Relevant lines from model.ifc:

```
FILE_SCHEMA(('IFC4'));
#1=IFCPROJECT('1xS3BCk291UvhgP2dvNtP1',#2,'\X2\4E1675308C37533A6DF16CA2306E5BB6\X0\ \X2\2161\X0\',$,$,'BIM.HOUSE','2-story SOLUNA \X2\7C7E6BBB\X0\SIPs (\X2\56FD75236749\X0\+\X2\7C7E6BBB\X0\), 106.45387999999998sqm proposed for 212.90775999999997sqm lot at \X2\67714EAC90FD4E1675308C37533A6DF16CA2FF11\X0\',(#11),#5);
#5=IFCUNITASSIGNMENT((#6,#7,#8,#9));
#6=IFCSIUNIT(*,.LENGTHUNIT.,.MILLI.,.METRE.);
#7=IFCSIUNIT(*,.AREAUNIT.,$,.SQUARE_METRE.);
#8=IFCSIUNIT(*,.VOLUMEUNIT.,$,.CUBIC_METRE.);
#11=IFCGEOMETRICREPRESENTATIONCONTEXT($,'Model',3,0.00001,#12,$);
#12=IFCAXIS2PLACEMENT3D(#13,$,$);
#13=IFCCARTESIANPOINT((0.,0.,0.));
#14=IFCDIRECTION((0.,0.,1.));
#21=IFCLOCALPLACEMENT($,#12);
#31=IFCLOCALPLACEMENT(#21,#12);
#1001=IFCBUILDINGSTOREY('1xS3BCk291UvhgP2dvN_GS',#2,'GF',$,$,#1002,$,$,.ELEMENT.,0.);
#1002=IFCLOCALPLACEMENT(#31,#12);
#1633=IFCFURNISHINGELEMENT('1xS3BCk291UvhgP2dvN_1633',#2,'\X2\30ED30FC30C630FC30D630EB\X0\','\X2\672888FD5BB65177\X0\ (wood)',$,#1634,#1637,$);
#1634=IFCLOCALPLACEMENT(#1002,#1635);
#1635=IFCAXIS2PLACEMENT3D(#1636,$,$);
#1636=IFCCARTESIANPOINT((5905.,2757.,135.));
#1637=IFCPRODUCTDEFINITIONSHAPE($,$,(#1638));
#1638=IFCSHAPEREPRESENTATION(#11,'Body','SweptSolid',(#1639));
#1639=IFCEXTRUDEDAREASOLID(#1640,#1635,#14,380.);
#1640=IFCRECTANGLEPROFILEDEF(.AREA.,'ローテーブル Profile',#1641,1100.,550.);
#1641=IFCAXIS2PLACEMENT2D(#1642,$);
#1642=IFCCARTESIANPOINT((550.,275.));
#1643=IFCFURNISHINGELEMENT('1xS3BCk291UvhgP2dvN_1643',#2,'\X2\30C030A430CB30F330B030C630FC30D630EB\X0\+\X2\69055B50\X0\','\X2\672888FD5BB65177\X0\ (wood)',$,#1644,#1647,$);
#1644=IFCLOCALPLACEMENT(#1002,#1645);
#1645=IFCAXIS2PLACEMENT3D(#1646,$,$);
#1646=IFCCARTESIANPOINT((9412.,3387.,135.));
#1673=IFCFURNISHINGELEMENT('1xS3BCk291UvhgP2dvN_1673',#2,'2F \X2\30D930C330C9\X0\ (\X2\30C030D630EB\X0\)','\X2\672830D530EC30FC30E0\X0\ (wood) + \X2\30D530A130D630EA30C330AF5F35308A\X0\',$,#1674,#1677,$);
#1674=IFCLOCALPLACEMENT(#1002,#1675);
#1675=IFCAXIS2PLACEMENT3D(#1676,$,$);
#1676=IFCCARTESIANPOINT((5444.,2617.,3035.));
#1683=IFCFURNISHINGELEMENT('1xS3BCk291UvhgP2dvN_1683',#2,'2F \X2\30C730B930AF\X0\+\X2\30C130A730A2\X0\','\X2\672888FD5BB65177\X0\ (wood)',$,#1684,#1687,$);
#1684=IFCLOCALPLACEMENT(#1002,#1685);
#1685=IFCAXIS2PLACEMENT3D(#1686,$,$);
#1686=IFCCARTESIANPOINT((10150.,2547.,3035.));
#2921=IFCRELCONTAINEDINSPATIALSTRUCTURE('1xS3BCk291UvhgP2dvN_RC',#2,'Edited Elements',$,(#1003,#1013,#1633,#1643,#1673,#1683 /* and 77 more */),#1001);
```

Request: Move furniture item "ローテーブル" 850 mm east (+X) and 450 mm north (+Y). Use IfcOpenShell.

```python
import ifcopenshell
import ifcopenshell.api.geometry
import ifcopenshell.util.placement

model = ifcopenshell.open("model.ifc")

item = model.by_id(1633)
matrix = ifcopenshell.util.placement.get_local_placement(item.ObjectPlacement)
matrix[0, 3] += 850.0
matrix[1, 3] += 450.0
ifcopenshell.api.geometry.edit_object_placement(model, product=item, matrix=matrix, is_si=False)

print(ifcopenshell.util.placement.get_local_placement(item.ObjectPlacement).round(3) + 0.0)

model.write("model_edited.ifc")
```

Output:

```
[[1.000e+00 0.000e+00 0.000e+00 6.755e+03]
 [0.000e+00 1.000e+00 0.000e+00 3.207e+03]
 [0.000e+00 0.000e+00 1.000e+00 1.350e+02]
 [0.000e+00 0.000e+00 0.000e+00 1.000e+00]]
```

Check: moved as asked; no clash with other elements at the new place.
